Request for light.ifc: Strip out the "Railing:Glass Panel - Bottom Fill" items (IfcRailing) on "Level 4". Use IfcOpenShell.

First a look at what the model holds.

```python
import ifcopenshell
import ifcopenshell.util.element

model = ifcopenshell.open("light.ifc")
print(model.schema)
storey = next(s for s in model.by_type("IfcBuildingStorey") if s.Name == "Level 4")
railings = [e for e in ifcopenshell.util.element.get_decomposition(storey) if e.is_a("IfcRailing")]
seen = {}
for e in railings:
    element_type = ifcopenshell.util.element.get_type(e)
    name = element_type.Name if element_type not in (None, e) else None
    seen[name] = seen.get(name, 0) + 1
for name, count in sorted(seen.items(), key=str):
    print(count, "x", name)
```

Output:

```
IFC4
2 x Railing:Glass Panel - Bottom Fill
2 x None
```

```python
import ifcopenshell
import ifcopenshell.api.root
import ifcopenshell.util.element

model = ifcopenshell.open("light.ifc")

storey = next(s for s in model.by_type("IfcBuildingStorey") if s.Name == "Level 4")
railings = [e for e in ifcopenshell.util.element.get_decomposition(storey) if e.is_a("IfcRailing")]
targets = [e for e in railings if (t := ifcopenshell.util.element.get_type(e)) not in (None, e) and t.Name == "Railing:Glass Panel - Bottom Fill"]

for e in targets:
    ifcopenshell.api.root.remove_product(model, product=e)
print(len(targets), "removed")

model.write("light_rev.ifc")
```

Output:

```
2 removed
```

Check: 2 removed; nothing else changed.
